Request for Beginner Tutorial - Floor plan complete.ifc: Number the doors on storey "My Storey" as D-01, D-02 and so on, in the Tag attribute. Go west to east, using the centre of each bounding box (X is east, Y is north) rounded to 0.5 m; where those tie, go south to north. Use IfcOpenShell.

First a look at what the model holds.

```python
import ifcopenshell
import ifcopenshell.util.element
import ifcopenshell.util.placement

model = ifcopenshell.open("Beginner Tutorial - Floor plan complete.ifc")
print(model.schema)
storey = next(s for s in model.by_type("IfcBuildingStorey") if s.Name == "My Storey")
doors = [e for e in ifcopenshell.util.element.get_decomposition(storey) if e.is_a("IfcDoor")]
for e in sorted(doors, key=lambda e: e.id()):
    origin = ifcopenshell.util.placement.get_local_placement(e.ObjectPlacement)[:3, 3]
    print(e.id(), e.Tag, e.Name, origin.round(2) + 0.0, sep=" | ")
```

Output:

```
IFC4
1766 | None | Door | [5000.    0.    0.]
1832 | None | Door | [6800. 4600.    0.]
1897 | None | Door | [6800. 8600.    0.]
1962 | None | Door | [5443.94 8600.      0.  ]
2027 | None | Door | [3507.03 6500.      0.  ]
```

```python
import ifcopenshell
import ifcopenshell.geom
import ifcopenshell.util.element
import ifcopenshell.util.shape

model = ifcopenshell.open("Beginner Tutorial - Floor plan complete.ifc")
settings = ifcopenshell.geom.settings()
settings.set("use-world-coords", True)


def centre(element):
    shape = ifcopenshell.geom.create_shape(settings, element)
    return ifcopenshell.util.shape.get_bbox_centroid(shape.geometry)


storey = next(s for s in model.by_type("IfcBuildingStorey") if s.Name == "My Storey")
doors = [e for e in ifcopenshell.util.element.get_decomposition(storey) if e.is_a("IfcDoor")]

# Insertion points can sit at a corner or the storey origin, so sort by the geometry (in metres).
centres = {e: centre(e) for e in doors}
doors.sort(key=lambda e: (round(centres[e][0] / 0.5), centres[e][1]))

for i, e in enumerate(doors, start=1):
    number = f"D-{i:02d}"
    e.Tag = number
    print(e.id(), number)

model.write("Beginner Tutorial - Floor plan complete_updated.ifc")
```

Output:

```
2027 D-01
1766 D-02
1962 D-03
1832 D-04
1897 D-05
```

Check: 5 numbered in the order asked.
